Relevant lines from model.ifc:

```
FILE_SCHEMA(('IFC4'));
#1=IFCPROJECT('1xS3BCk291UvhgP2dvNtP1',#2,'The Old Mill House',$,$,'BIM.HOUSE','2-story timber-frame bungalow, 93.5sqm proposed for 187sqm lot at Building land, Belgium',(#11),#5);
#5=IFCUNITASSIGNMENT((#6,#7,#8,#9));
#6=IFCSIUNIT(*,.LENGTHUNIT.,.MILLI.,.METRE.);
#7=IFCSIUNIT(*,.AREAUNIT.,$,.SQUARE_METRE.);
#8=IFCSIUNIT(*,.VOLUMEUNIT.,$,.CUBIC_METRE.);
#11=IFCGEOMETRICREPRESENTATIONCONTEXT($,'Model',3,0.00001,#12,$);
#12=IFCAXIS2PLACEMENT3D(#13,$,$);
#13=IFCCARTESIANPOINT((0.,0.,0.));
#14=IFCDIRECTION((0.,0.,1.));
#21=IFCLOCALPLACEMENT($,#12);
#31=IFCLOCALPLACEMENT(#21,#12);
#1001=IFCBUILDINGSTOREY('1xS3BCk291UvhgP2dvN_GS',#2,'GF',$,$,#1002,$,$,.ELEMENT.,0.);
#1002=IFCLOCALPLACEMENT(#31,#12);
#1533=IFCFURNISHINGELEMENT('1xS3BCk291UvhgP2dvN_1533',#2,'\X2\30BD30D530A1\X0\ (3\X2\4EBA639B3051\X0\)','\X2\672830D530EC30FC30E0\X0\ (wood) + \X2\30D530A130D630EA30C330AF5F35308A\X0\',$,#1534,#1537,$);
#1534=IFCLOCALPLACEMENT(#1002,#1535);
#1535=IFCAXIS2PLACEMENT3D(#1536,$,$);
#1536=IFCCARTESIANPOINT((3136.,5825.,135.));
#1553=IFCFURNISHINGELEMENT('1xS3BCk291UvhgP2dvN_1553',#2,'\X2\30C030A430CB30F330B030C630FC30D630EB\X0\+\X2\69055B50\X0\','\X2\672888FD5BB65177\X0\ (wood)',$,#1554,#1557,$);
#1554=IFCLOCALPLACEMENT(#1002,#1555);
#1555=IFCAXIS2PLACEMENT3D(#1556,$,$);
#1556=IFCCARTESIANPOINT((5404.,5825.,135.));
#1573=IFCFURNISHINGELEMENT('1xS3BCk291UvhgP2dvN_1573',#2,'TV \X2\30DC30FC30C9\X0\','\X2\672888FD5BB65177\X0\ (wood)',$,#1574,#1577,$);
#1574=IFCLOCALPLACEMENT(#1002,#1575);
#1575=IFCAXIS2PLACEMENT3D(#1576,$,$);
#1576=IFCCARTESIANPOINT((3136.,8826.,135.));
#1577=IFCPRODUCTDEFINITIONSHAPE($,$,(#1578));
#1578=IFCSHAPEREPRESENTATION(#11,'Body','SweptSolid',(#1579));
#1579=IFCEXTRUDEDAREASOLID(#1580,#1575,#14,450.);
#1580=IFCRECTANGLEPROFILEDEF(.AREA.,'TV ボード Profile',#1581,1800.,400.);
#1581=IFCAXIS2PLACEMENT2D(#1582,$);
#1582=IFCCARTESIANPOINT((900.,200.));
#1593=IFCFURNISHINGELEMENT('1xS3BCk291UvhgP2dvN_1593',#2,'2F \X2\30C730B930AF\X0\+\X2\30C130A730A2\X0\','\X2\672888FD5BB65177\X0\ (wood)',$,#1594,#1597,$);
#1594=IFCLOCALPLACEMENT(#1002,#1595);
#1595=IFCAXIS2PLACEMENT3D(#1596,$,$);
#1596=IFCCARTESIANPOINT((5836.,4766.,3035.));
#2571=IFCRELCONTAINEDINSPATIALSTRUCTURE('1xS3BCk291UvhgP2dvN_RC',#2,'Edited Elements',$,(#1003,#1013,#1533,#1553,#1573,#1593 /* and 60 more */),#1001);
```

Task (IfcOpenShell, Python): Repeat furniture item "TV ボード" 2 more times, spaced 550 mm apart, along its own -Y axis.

```python
import ifcopenshell
import ifcopenshell.api.geometry
import ifcopenshell.api.root
import ifcopenshell.util.element
import ifcopenshell.util.placement
import ifcopenshell.util.unit

model = ifcopenshell.open("model.ifc")
unit_scale = ifcopenshell.util.unit.calculate_unit_scale(model)


def reuse_history(source, copy):
    """copy_class also copies each property set's owner history, people and application; keep the originals."""
    for rel in copy.IsDefinedBy:
        if rel.is_a("IfcRelDefinesByProperties") and (history := rel.RelatingPropertyDefinition.OwnerHistory):
            rel.RelatingPropertyDefinition.OwnerHistory = source.OwnerHistory
            ifcopenshell.util.element.remove_deep2(model, history)


source = model.by_guid("1xS3BCk291UvhgP2dvN_1573")
base = ifcopenshell.util.placement.get_local_placement(source.ObjectPlacement)
step = -base[:3, 1] * 0.55 / unit_scale

for i in range(1, 3):
    copy = ifcopenshell.api.root.copy_class(model, product=source)
    copy.Representation = ifcopenshell.util.element.copy_deep(
        model, source.Representation, exclude=["IfcGeometricRepresentationContext", "IfcRepresentationMap"]
    )
    reuse_history(source, copy)
    matrix = base.copy()
    matrix[:3, 3] += i * step
    print("added at", matrix[:3, 3].round(3) + 0.0)
    ifcopenshell.api.geometry.edit_object_placement(model, product=copy, matrix=matrix, is_si=False)

model.write("model_v2.ifc")
```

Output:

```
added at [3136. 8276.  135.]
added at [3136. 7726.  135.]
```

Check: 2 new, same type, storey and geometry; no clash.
